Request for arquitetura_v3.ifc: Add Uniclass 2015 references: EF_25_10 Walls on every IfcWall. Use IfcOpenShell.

First a look at what the model holds.

```python
import ifcopenshell

model = ifcopenshell.open("arquitetura_v3.ifc")
print(model.schema)
print("classifications:", [c.Name for c in model.by_type("IfcClassification")])
for ifc_class in ("IfcDoor", "IfcRoof", "IfcStair", "IfcWall", "IfcWindow"):
    print(ifc_class, len(model.by_type(ifc_class)))
```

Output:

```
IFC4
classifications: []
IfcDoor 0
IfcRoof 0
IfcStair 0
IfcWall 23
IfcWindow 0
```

```python
import ifcopenshell
import ifcopenshell.api.classification

model = ifcopenshell.open("arquitetura_v3.ifc")

system = ifcopenshell.api.classification.add_classification(model, classification="Uniclass 2015")

codes = {
    "IfcWall": ("EF_25_10", "Walls"),
}
for ifc_class, (code, name) in codes.items():
    products = model.by_type(ifc_class)
    ifcopenshell.api.classification.add_reference(
        model, products=products, classification=system, identification=code, name=name
    )
    print(code, len(products))

model.write("arquitetura_v3_rev.ifc")
```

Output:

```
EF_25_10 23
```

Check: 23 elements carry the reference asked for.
